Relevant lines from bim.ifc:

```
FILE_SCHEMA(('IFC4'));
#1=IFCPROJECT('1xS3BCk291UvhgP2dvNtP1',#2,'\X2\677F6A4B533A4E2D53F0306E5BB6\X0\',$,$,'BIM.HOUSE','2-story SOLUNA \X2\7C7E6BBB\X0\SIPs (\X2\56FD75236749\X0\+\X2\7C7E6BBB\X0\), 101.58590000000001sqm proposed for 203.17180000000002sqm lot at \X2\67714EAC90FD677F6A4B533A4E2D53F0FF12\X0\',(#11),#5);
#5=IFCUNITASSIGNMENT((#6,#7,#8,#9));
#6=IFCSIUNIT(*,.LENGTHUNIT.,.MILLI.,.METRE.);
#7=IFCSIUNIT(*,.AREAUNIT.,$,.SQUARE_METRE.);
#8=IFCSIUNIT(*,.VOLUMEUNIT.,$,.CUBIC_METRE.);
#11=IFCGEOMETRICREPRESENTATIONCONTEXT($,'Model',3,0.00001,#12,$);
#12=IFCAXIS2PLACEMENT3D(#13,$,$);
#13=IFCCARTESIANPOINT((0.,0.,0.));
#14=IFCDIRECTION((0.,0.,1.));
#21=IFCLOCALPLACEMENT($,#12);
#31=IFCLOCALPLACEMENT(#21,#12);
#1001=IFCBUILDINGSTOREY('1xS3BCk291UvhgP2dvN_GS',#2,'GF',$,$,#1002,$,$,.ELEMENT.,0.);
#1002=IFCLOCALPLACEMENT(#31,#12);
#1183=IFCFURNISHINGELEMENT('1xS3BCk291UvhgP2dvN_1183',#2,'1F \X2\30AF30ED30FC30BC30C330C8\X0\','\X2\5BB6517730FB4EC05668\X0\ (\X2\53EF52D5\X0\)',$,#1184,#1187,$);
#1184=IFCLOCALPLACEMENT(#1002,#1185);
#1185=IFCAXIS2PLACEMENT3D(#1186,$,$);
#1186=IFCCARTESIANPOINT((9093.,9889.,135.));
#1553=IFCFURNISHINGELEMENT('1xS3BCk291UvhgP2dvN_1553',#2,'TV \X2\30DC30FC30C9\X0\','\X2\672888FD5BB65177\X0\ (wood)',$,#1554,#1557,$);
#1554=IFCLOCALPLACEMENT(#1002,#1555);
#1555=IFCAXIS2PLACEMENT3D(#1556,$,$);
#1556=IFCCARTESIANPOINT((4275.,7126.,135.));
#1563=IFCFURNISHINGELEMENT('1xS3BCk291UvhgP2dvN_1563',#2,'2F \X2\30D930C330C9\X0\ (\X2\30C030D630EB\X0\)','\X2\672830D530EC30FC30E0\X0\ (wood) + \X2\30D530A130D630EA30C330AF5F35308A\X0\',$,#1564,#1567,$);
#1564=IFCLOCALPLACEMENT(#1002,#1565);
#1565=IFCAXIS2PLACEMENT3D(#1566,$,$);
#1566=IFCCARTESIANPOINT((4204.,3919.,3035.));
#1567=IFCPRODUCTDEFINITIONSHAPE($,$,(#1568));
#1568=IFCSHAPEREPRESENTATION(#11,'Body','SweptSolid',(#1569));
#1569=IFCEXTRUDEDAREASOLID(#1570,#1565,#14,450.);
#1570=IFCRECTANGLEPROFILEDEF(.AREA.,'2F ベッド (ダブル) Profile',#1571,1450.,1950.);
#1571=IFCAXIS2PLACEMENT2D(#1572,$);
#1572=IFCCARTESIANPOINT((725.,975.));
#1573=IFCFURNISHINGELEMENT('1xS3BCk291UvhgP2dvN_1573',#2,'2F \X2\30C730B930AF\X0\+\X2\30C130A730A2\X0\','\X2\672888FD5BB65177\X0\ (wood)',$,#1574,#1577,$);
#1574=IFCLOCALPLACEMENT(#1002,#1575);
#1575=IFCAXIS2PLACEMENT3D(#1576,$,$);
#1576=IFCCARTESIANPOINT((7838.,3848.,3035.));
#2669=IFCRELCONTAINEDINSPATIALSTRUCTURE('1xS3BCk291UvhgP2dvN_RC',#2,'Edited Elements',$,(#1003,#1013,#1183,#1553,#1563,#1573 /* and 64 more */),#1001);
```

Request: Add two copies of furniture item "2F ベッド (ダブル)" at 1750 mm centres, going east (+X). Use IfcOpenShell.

```python
import numpy as np
import ifcopenshell
import ifcopenshell.api.geometry
import ifcopenshell.api.root
import ifcopenshell.util.element
import ifcopenshell.util.placement

model = ifcopenshell.open("bim.ifc")


def reuse_history(source, copy):
    """copy_class also copies each property set's owner history, people and application; keep the originals."""
    for rel in copy.IsDefinedBy:
        if rel.is_a("IfcRelDefinesByProperties") and (history := rel.RelatingPropertyDefinition.OwnerHistory):
            rel.RelatingPropertyDefinition.OwnerHistory = source.OwnerHistory
            ifcopenshell.util.element.remove_deep2(model, history)


source = model.by_guid("1xS3BCk291UvhgP2dvN_1563")
base = ifcopenshell.util.placement.get_local_placement(source.ObjectPlacement)
step = np.array([1.0, 0.0, 0.0]) * 1750.0

for i in range(1, 3):
    copy = ifcopenshell.api.root.copy_class(model, product=source)
    copy.Representation = ifcopenshell.util.element.copy_deep(
        model, source.Representation, exclude=["IfcGeometricRepresentationContext", "IfcRepresentationMap"]
    )
    reuse_history(source, copy)
    matrix = base.copy()
    matrix[:3, 3] += i * step
    print("added at", matrix[:3, 3].round(3) + 0.0)
    ifcopenshell.api.geometry.edit_object_placement(model, product=copy, matrix=matrix, is_si=False)

model.write("bim_updated.ifc")
```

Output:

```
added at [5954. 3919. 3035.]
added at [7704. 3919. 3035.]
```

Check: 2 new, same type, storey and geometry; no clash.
